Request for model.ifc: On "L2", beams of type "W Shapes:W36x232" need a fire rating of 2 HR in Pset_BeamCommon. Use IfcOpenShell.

First a look at what the model holds.

```python
import ifcopenshell
import ifcopenshell.util.element

model = ifcopenshell.open("model.ifc")
print(model.schema)
storey = next(s for s in model.by_type("IfcBuildingStorey") if s.Name == "L2")
beams = [e for e in ifcopenshell.util.element.get_decomposition(storey) if e.is_a("IfcBeam")]
seen = {}
for e in beams:
    element_type = ifcopenshell.util.element.get_type(e)
    key = (element_type.Name if element_type != e and element_type else None, ifcopenshell.util.element.get_pset(e, "Pset_BeamCommon", "FireRating"))
    seen[key] = seen.get(key, 0) + 1
for (name, value), count in sorted(seen.items(), key=str):
    print(count, "x", name, "|", value)
```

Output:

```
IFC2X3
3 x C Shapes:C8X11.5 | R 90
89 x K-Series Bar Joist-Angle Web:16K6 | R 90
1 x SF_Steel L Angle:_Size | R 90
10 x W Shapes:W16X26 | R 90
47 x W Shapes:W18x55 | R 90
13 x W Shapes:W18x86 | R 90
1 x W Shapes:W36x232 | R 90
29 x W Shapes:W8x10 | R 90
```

```python
import ifcopenshell
import ifcopenshell.api.pset
import ifcopenshell.util.element

model = ifcopenshell.open("model.ifc")

storey = next(s for s in model.by_type("IfcBuildingStorey") if s.Name == "L2")
beams = [e for e in ifcopenshell.util.element.get_decomposition(storey) if e.is_a("IfcBeam")]

count = 0
for e in beams:
    element_type = ifcopenshell.util.element.get_type(e)
    if element_type in (None, e) or element_type.Name != "W Shapes:W36x232":
        continue
    # add_pset returns the element's existing set when there is one.
    pset = ifcopenshell.api.pset.add_pset(model, product=e, name="Pset_BeamCommon")
    ifcopenshell.api.pset.edit_pset(model, pset=pset, properties={"FireRating": "2 HR"})
    count += 1

print(count, "beams updated")

model.write("model_v2.ifc")
```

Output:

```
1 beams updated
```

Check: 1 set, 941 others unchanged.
